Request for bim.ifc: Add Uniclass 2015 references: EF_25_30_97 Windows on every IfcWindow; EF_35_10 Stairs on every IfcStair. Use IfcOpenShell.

First a look at what the model holds.

```python
import ifcopenshell

model = ifcopenshell.open("bim.ifc")
print(model.schema)
print("classifications:", [c.Name for c in model.by_type("IfcClassification")])
for ifc_class in ("IfcDoor", "IfcRoof", "IfcStair", "IfcWall", "IfcWindow"):
    print(ifc_class, len(model.by_type(ifc_class)))
```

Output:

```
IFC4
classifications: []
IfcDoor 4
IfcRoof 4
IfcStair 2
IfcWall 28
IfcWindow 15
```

```python
import ifcopenshell
import ifcopenshell.api.classification

model = ifcopenshell.open("bim.ifc")

system = ifcopenshell.api.classification.add_classification(model, classification="Uniclass 2015")

codes = {
    "IfcWindow": ("EF_25_30_97", "Windows"),
    "IfcStair": ("EF_35_10", "Stairs"),
}
for ifc_class, (code, name) in codes.items():
    products = model.by_type(ifc_class)
    ifcopenshell.api.classification.add_reference(
        model, products=products, classification=system, identification=code, name=name
    )
    print(code, len(products))

model.write("bim_updated.ifc")
```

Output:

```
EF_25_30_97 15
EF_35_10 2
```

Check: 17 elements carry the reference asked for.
